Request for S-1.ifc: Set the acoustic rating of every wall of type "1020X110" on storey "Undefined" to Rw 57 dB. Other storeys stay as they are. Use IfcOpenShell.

First a look at what the model holds.

```python
import ifcopenshell
import ifcopenshell.util.element

model = ifcopenshell.open("S-1.ifc")
print(model.schema)
storey = next(s for s in model.by_type("IfcBuildingStorey") if s.Name == "Undefined")
walls = [e for e in ifcopenshell.util.element.get_decomposition(storey) if e.is_a("IfcWall")]
seen = {}
for e in walls:
    element_type = ifcopenshell.util.element.get_type(e)
    key = (element_type.Name if element_type != e and element_type else None, ifcopenshell.util.element.get_pset(e, "Pset_WallCommon", "AcousticRating"))
    seen[key] = seen.get(key, 0) + 1
for (name, value), count in sorted(seen.items(), key=str):
    print(count, "x", name, "|", value)
```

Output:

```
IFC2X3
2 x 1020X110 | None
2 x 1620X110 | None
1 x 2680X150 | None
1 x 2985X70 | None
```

```python
import ifcopenshell
import ifcopenshell.api.pset
import ifcopenshell.util.element

model = ifcopenshell.open("S-1.ifc")

storey = next(s for s in model.by_type("IfcBuildingStorey") if s.Name == "Undefined")
walls = [e for e in ifcopenshell.util.element.get_decomposition(storey) if e.is_a("IfcWall")]

count = 0
for e in walls:
    element_type = ifcopenshell.util.element.get_type(e)
    if element_type in (None, e) or element_type.Name != "1020X110":
        continue
    found = ifcopenshell.util.element.get_pset(e, "Pset_WallCommon", should_inherit=False)
    if found:
        pset = model.by_id(found["id"])
        if len(ifcopenshell.util.element.get_elements_by_pset(pset)) > 1:
            pset = ifcopenshell.api.pset.unshare_pset(model, products=[e], pset=pset)[0]
    else:
        pset = ifcopenshell.api.pset.add_pset(model, product=e, name="Pset_WallCommon")
    ifcopenshell.api.pset.edit_pset(model, pset=pset, properties={"AcousticRating": "Rw 57 dB"})
    count += 1

print(count, "walls updated")

model.write("S-1_updated.ifc")
```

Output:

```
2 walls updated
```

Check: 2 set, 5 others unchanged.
